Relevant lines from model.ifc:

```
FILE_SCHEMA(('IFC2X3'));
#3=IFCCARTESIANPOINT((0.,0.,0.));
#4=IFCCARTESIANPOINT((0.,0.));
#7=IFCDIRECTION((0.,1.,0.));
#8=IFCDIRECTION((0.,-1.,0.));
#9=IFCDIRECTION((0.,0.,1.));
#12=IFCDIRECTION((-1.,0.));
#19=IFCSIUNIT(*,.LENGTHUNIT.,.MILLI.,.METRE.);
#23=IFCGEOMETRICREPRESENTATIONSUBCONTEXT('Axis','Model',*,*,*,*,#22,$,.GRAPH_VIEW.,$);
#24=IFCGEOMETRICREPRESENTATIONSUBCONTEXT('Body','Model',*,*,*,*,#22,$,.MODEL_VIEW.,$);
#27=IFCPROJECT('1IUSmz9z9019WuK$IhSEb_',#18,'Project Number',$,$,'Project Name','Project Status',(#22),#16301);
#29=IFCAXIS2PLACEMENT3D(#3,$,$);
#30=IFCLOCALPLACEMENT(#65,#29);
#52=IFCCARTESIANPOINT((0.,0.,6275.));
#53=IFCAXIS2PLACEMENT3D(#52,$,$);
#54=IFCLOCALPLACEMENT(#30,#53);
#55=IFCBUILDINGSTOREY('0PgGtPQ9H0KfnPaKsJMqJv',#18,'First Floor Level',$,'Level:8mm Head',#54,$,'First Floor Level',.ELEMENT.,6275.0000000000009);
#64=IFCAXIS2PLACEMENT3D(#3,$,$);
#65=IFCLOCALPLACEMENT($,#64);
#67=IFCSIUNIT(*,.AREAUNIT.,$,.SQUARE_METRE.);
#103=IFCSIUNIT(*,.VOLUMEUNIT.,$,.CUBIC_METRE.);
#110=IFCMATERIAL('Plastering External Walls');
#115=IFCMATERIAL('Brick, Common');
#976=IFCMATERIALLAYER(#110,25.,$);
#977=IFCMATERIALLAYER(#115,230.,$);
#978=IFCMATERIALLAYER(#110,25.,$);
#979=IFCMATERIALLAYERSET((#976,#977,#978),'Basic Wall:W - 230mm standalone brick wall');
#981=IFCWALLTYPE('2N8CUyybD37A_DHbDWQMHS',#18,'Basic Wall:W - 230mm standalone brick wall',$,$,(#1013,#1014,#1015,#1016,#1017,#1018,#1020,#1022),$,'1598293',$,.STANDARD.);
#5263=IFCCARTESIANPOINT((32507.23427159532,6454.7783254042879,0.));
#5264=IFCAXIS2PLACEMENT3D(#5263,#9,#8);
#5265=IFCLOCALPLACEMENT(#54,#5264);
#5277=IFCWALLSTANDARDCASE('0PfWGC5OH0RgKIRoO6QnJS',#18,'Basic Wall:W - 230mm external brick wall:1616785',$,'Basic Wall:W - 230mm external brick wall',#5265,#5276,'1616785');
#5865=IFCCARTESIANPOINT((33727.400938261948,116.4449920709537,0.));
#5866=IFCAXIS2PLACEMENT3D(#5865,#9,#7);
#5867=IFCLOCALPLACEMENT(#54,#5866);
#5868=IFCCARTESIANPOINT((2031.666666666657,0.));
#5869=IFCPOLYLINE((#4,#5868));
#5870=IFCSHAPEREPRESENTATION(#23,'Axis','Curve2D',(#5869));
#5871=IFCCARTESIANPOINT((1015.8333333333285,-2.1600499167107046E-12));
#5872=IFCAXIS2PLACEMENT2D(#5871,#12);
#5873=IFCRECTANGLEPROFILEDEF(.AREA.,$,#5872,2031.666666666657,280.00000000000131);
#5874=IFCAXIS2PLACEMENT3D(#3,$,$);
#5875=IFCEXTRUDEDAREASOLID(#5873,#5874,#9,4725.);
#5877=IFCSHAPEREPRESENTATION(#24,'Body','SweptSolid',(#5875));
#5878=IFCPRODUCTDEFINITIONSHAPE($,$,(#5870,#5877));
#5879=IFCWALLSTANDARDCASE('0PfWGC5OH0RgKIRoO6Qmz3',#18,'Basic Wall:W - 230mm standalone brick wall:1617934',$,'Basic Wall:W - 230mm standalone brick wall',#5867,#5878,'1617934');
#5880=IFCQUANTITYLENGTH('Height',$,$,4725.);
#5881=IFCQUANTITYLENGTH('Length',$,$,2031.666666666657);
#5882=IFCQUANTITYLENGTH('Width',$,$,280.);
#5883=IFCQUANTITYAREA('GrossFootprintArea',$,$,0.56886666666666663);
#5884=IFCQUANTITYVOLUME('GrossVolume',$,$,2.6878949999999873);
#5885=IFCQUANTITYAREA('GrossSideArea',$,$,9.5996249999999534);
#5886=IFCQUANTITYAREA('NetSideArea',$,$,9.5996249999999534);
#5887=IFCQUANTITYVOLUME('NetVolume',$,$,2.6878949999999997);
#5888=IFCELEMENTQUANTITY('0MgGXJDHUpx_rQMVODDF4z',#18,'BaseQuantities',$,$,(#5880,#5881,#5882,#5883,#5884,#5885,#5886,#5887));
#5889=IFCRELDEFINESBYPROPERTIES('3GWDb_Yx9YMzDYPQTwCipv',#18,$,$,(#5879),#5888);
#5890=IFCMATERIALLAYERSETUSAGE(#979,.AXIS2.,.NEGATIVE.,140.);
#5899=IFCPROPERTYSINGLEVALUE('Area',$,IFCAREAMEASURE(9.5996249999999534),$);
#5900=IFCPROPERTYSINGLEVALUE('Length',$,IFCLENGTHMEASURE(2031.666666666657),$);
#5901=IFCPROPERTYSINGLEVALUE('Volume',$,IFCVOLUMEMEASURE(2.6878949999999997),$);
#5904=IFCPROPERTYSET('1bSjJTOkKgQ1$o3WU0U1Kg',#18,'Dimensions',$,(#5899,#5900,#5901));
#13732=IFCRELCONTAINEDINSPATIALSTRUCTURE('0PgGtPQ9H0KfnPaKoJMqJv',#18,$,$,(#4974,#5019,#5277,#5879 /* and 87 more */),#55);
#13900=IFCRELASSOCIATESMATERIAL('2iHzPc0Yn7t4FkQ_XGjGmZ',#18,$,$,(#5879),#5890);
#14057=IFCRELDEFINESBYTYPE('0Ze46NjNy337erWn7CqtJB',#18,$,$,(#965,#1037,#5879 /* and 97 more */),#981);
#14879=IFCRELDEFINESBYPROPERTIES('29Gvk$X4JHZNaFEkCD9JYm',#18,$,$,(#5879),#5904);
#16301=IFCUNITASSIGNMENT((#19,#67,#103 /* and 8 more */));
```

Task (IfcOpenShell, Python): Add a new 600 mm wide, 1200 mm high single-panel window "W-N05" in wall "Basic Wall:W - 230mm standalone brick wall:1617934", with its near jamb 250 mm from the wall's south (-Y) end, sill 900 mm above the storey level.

```python
import numpy as np
import ifcopenshell
import ifcopenshell.api.feature
import ifcopenshell.api.geometry
import ifcopenshell.api.pset
import ifcopenshell.api.root
import ifcopenshell.api.spatial
import ifcopenshell.api.type
import ifcopenshell.geom
import ifcopenshell.util.element
import ifcopenshell.util.placement
import ifcopenshell.util.representation
import ifcopenshell.util.shape
import ifcopenshell.util.unit

model = ifcopenshell.open("model.ifc")
unit_scale = ifcopenshell.util.unit.calculate_unit_scale(model)
area_scale = ifcopenshell.util.unit.calculate_unit_scale(model, "AREAUNIT")
volume_scale = ifcopenshell.util.unit.calculate_unit_scale(model, "VOLUMEUNIT")
settings = ifcopenshell.geom.settings()


def volume(element):
    """Net volume in cubic metres, openings subtracted."""
    shape = ifcopenshell.geom.create_shape(settings, element)
    return ifcopenshell.util.shape.get_volume(shape.geometry)


wall = model.by_guid("0PfWGC5OH0RgKIRoO6Qmz3")
storey = ifcopenshell.util.element.get_container(wall, ifc_class="IfcBuildingStorey")
context = ifcopenshell.util.representation.get_context(model, "Model", "Body", "MODEL_VIEW")
before = volume(wall)

width, height, from_end, sill = 0.6, 1.2, 0.25, 0.9  # metres

# The wall runs along its own X axis, and the end named is its -X end.
wall_shape = ifcopenshell.geom.create_shape(settings, wall)
x, y, z = ifcopenshell.util.shape.get_vertices(wall_shape.geometry).T
start = x.min() + from_end
face, thickness = float(y.min()), float(y.max() - y.min())
wall_matrix = ifcopenshell.util.placement.get_local_placement(wall.ObjectPlacement)
level = ifcopenshell.util.placement.get_local_placement(storey.ObjectPlacement)[2, 3]


def in_wall(x, y):
    """Placement at x, y metres in the wall's axes, at sill height."""
    matrix = wall_matrix.copy()
    matrix[:, 3] = wall_matrix @ np.array([x / unit_scale, y / unit_scale, 0.0, 1.0])
    matrix[2, 3] = level + sill / unit_scale
    return matrix


# Opening: a box that overshoots both wall faces by 50 mm.
opening = ifcopenshell.api.root.create_entity(model, ifc_class="IfcOpeningElement")
box = ifcopenshell.api.geometry.add_wall_representation(
    model, context=context, length=width, height=height, thickness=thickness + 0.1
)
ifcopenshell.api.geometry.assign_representation(model, product=opening, representation=box)
ifcopenshell.api.geometry.edit_object_placement(model, product=opening, matrix=in_wall(start, face - 0.05), is_si=False)
ifcopenshell.api.feature.add_feature(model, feature=opening, element=wall)

window = ifcopenshell.api.root.create_entity(model, ifc_class="IfcWindow", name="W-N05")
window.OverallWidth, window.OverallHeight = width / unit_scale, height / unit_scale
body = ifcopenshell.api.geometry.add_window_representation(
    model,
    context=context,
    overall_width=window.OverallWidth,
    overall_height=window.OverallHeight,
    partition_type="SINGLE_PANEL",
)
ifcopenshell.api.geometry.assign_representation(model, product=window, representation=body)
ifcopenshell.api.spatial.assign_container(model, products=[window], relating_structure=storey)
fills = ifcopenshell.api.feature.add_filling(model, opening=opening, element=window)
fills.OwnerHistory = window.OwnerHistory  # required in IFC2X3

# IFC2X3 keeps the operation on the window style.
style = ifcopenshell.api.root.create_entity(model, ifc_class="IfcWindowStyle", name="W-N05")
style.OperationType, style.ConstructionType = "SINGLE_PANEL", "NOTDEFINED"
style.ParameterTakesPrecedence = style.Sizeable = False
ifcopenshell.api.type.assign_type(model, related_objects=[window], relating_type=style)

# Centre the window in the wall's thickness.
ifcopenshell.api.geometry.edit_object_placement(model, product=window, matrix=in_wall(start, face), is_si=False)
window_shape = ifcopenshell.geom.create_shape(settings, window)
depth = ifcopenshell.util.shape.get_vertices(window_shape.geometry)[:, 1]
offset = face + thickness / 2 - (depth.min() + depth.max()) / 2
ifcopenshell.api.geometry.edit_object_placement(model, product=window, matrix=in_wall(start, offset), is_si=False)

after = volume(wall)

# Update the wall's stored quantities.
qto = model.by_id(ifcopenshell.util.element.get_pset(wall, "BaseQuantities", should_inherit=False)["id"])
ifcopenshell.api.pset.edit_qto(model, qto=qto, properties={
    "NetSideArea": after / thickness / area_scale,
    "NetVolume": after / volume_scale,
})
pset = model.by_id(ifcopenshell.util.element.get_pset(wall, "Dimensions", should_inherit=False)["id"])
ifcopenshell.api.pset.edit_pset(model, pset=pset, properties={
    "Area": model.create_entity("IfcAreaMeasure", after / thickness / area_scale),
    "Volume": model.create_entity("IfcVolumeMeasure", after / volume_scale),
})

print(f"wall volume {before:.3f} -> {after:.3f} m3")

model.write("model_edited.ifc")
```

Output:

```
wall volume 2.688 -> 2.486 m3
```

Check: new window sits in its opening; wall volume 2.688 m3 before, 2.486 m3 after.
